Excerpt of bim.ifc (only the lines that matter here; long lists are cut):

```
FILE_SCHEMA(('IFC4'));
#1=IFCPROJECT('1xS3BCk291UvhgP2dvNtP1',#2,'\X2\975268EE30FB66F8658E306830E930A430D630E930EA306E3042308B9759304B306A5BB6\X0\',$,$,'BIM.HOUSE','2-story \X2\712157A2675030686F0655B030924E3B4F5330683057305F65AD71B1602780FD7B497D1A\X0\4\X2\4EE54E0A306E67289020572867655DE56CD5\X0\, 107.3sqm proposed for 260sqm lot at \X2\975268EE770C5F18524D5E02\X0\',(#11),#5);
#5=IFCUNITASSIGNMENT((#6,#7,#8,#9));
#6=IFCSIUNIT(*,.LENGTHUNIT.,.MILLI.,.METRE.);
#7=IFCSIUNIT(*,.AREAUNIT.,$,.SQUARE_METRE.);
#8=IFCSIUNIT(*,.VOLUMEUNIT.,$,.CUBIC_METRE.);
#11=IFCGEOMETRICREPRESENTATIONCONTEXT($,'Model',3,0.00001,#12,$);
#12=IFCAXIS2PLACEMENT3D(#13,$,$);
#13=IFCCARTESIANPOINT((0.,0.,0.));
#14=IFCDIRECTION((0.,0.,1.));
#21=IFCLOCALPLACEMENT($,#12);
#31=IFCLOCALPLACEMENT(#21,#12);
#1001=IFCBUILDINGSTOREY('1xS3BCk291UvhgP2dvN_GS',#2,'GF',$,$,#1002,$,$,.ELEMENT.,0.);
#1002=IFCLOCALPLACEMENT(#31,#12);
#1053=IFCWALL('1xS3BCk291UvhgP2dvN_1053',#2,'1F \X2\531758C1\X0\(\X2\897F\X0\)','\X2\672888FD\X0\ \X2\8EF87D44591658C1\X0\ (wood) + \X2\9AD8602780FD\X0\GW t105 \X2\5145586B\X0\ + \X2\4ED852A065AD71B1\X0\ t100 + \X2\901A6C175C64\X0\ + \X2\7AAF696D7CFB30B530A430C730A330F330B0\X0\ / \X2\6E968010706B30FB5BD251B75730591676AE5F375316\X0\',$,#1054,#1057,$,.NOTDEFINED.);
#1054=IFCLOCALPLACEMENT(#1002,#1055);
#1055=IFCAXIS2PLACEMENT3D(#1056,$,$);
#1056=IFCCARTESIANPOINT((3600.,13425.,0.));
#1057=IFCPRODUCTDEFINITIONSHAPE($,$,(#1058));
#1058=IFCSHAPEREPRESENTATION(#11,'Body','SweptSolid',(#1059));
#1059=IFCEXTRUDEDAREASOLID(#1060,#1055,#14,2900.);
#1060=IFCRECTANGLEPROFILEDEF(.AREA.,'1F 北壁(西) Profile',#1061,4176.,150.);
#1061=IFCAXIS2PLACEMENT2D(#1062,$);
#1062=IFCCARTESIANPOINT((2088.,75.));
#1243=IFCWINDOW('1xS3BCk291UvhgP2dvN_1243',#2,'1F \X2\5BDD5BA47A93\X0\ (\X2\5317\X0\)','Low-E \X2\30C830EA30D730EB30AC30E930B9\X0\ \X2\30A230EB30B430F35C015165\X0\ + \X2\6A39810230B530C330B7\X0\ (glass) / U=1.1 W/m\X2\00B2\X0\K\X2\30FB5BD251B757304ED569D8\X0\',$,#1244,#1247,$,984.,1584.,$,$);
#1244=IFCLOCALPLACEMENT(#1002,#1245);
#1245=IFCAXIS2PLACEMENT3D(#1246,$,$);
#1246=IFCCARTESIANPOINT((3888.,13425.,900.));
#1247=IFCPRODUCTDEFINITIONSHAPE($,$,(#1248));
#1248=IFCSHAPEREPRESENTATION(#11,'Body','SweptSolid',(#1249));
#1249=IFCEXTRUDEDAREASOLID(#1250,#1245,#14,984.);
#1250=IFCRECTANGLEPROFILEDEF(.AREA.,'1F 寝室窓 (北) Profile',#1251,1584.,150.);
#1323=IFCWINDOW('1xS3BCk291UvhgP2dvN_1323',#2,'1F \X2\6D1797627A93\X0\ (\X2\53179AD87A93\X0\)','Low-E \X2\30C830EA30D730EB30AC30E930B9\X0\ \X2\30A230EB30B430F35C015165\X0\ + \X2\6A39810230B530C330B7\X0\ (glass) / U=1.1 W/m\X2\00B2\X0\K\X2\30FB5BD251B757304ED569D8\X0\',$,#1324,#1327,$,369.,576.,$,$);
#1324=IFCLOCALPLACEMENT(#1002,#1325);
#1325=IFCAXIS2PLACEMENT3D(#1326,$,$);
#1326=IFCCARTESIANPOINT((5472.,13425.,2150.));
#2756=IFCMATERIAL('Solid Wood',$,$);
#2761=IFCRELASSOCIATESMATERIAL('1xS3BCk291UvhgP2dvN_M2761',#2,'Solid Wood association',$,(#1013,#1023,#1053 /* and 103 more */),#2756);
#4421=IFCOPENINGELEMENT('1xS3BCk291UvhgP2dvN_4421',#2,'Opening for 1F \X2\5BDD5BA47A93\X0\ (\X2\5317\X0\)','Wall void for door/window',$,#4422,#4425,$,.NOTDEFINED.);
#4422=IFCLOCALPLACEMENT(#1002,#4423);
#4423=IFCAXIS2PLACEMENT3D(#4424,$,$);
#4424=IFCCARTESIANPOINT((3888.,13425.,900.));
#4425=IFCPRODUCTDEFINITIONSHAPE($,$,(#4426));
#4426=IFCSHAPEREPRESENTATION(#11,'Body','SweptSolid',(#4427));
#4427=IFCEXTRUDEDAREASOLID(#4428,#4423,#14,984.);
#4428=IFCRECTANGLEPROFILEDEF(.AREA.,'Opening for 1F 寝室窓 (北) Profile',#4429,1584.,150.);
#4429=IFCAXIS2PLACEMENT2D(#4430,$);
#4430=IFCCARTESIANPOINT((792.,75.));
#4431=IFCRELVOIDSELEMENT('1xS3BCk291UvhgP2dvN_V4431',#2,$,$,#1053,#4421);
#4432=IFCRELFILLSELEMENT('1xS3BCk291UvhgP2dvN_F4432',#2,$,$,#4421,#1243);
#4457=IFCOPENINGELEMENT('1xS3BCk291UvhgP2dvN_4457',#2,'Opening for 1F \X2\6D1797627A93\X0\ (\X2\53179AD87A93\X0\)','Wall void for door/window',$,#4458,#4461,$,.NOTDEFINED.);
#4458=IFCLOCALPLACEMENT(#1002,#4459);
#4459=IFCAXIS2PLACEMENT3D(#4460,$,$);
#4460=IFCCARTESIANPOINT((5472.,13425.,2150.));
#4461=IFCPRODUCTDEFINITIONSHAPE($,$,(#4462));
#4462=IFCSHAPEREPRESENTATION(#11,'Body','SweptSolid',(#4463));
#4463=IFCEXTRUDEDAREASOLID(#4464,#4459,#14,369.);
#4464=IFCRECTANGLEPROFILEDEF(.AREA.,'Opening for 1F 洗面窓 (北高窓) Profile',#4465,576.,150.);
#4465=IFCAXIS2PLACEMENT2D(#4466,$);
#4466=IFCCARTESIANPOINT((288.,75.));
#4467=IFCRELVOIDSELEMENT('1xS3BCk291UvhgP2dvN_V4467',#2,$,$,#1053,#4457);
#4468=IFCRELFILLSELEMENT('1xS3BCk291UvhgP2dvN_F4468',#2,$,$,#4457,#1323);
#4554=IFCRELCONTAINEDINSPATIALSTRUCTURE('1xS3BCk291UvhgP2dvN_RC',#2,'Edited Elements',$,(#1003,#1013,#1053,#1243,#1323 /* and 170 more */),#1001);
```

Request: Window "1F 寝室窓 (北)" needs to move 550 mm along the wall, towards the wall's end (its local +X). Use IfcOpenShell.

```python
import ifcopenshell
import ifcopenshell.api.geometry
import ifcopenshell.util.placement

model = ifcopenshell.open("bim.ifc")

window = model.by_guid("1xS3BCk291UvhgP2dvN_1243")
opening = window.FillsVoids[0].RelatingOpeningElement
wall = opening.VoidsElements[0].RelatingBuildingElement

wall_matrix = ifcopenshell.util.placement.get_local_placement(wall.ObjectPlacement)
shift = wall_matrix[:3, 0] * 550.0
before = ifcopenshell.util.placement.get_local_placement(window.ObjectPlacement)[:3, 3].copy()

# The window is not placed relative to its opening, so move both.
for product in (opening, window):
    matrix = ifcopenshell.util.placement.get_local_placement(product.ObjectPlacement)
    matrix[:3, 3] += shift
    ifcopenshell.api.geometry.edit_object_placement(model, product=product, matrix=matrix, is_si=False)

after = ifcopenshell.util.placement.get_local_placement(window.ObjectPlacement)[:3, 3]
print("window moved by", (after - before).round(3) + 0.0)

model.write("bim_updated.ifc")
```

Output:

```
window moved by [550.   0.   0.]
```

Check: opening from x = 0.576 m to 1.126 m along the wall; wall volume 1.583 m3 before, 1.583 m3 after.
